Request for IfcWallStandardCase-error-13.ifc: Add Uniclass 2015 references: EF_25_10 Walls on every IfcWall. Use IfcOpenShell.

First a look at what the model holds.

```python
import ifcopenshell

model = ifcopenshell.open("IfcWallStandardCase-error-13.ifc")
print(model.schema)
print("classifications:", [c.Name for c in model.by_type("IfcClassification")])
for ifc_class in ("IfcDoor", "IfcRoof", "IfcStair", "IfcWall", "IfcWindow"):
    print(ifc_class, len(model.by_type(ifc_class)))
```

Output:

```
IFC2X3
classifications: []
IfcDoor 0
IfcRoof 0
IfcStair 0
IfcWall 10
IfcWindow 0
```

```python
import ifcopenshell
import ifcopenshell.api.classification

model = ifcopenshell.open("IfcWallStandardCase-error-13.ifc")

# IFC2X3 requires Source and Edition and has no link from the project to the system.
system = model.create_entity("IfcClassification", Source="NBS", Edition="2015", Name="Uniclass 2015")

codes = {
    "IfcWall": ("EF_25_10", "Walls"),
}
for ifc_class, (code, name) in codes.items():
    products = model.by_type(ifc_class)
    ifcopenshell.api.classification.add_reference(
        model, products=products, classification=system, identification=code, name=name
    )
    print(code, len(products))

model.write("IfcWallStandardCase-error-13_v2.ifc")
```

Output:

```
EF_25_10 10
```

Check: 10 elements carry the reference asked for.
